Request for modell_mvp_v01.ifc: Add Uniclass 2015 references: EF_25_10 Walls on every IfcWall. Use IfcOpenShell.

First a look at what the model holds.

```python
import ifcopenshell

model = ifcopenshell.open("modell_mvp_v01.ifc")
print(model.schema)
print("classifications:", [c.Name for c in model.by_type("IfcClassification")])
for ifc_class in ("IfcDoor", "IfcRoof", "IfcStair", "IfcWall", "IfcWindow"):
    print(ifc_class, len(model.by_type(ifc_class)))
```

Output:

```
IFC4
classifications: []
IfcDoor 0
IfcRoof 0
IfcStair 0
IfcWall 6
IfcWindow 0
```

```python
import ifcopenshell
import ifcopenshell.api.classification

model = ifcopenshell.open("modell_mvp_v01.ifc")

system = ifcopenshell.api.classification.add_classification(model, classification="Uniclass 2015")

codes = {
    "IfcWall": ("EF_25_10", "Walls"),
}
for ifc_class, (code, name) in codes.items():
    products = model.by_type(ifc_class)
    ifcopenshell.api.classification.add_reference(
        model, products=products, classification=system, identification=code, name=name
    )
    print(code, len(products))

model.write("modell_mvp_v01_updated.ifc")
```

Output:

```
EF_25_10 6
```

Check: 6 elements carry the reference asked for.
